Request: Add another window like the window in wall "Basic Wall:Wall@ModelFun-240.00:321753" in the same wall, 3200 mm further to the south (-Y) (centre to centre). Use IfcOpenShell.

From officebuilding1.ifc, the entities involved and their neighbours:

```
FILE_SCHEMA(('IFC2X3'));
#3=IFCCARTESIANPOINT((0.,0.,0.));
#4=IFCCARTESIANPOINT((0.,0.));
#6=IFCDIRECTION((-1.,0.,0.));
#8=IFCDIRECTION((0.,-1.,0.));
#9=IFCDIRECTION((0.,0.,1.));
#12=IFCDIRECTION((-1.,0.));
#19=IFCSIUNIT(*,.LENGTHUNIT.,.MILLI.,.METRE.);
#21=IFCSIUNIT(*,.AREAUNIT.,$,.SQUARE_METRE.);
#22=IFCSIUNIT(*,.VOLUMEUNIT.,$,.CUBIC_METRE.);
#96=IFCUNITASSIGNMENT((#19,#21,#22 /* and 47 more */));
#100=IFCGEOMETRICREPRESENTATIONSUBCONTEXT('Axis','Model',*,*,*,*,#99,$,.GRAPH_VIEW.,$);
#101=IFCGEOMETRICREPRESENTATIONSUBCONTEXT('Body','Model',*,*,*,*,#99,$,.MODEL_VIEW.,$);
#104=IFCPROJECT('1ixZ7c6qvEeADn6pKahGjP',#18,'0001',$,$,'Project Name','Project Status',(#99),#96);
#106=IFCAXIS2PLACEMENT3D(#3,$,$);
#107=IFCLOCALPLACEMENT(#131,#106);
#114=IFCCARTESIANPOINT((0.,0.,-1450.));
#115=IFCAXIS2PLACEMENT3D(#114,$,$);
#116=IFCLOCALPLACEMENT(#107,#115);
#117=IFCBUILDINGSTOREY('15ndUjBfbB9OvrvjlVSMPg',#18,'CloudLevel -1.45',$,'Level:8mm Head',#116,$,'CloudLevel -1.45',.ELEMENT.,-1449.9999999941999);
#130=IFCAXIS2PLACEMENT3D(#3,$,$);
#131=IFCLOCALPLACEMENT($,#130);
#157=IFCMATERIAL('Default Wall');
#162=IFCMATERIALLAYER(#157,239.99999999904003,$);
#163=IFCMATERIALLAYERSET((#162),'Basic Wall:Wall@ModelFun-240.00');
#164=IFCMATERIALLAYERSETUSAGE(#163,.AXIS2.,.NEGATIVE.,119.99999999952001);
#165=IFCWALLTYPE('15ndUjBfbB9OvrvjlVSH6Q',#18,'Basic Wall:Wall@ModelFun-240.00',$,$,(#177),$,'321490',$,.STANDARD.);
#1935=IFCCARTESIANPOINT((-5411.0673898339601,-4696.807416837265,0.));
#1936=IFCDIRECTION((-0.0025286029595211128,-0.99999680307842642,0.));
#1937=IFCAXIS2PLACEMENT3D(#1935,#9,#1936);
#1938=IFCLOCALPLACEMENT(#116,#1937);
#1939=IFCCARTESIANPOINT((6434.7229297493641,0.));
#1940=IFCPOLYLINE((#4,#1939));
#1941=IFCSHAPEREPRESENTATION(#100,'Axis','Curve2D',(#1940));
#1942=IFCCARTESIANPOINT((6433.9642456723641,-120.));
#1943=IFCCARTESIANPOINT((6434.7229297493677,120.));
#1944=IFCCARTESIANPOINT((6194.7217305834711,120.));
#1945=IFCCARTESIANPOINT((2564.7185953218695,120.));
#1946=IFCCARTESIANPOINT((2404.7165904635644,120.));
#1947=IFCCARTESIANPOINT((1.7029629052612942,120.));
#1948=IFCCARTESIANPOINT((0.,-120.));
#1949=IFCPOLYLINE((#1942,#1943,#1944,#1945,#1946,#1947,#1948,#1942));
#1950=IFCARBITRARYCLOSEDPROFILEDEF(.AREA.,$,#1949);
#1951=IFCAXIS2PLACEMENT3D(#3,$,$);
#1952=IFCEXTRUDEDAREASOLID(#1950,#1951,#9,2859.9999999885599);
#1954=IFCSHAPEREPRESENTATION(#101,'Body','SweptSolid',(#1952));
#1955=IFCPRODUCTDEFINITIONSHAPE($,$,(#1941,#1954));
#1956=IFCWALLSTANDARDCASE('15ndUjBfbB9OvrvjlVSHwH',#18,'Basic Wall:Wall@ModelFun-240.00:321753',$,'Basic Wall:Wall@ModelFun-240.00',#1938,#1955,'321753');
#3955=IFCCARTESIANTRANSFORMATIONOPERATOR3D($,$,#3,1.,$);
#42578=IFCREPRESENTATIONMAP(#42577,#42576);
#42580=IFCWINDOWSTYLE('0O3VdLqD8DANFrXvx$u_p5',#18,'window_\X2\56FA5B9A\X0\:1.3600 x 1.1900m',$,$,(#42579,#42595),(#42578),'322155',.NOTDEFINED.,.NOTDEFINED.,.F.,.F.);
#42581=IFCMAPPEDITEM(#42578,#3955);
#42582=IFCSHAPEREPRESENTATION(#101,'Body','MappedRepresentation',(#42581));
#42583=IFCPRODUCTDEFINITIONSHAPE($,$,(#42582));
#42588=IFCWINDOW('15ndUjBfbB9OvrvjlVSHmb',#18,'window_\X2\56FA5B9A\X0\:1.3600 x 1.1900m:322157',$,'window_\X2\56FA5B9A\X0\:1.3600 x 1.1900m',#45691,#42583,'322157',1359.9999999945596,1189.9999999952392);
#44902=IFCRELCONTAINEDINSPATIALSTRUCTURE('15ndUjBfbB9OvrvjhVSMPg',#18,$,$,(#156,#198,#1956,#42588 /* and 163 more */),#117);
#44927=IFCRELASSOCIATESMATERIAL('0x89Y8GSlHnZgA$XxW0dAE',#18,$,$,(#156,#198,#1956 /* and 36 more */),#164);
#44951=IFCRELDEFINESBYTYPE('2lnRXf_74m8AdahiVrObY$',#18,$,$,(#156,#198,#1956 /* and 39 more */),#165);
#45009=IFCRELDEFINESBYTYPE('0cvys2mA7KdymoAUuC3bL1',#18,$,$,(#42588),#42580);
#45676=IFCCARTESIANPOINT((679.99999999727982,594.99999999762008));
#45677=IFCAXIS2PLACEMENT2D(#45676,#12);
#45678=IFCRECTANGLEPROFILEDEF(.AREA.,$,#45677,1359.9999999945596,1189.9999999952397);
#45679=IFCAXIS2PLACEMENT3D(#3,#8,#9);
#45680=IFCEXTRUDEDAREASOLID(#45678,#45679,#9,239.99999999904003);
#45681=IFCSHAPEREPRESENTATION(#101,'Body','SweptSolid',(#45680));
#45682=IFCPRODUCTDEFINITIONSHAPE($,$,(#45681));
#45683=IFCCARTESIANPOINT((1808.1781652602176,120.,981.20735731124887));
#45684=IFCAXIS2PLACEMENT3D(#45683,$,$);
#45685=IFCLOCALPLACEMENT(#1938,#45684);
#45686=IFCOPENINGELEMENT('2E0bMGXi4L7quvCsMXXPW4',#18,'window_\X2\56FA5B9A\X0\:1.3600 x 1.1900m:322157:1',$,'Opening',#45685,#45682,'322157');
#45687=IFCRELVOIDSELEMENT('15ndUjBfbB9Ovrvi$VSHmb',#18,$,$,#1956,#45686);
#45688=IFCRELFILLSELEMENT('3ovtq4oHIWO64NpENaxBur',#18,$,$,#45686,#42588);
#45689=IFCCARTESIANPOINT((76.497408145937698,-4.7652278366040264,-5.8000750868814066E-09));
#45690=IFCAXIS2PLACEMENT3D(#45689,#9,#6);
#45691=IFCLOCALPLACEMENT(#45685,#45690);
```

```python
import ifcopenshell
import ifcopenshell.api.feature
import ifcopenshell.api.geometry
import ifcopenshell.api.root
import ifcopenshell.geom
import ifcopenshell.util.element
import ifcopenshell.util.placement
import ifcopenshell.util.shape
import ifcopenshell.util.unit

model = ifcopenshell.open("officebuilding1.ifc")
unit_scale = ifcopenshell.util.unit.calculate_unit_scale(model)
settings = ifcopenshell.geom.settings()


def volume(element):
    """Net volume in cubic metres, openings subtracted."""
    shape = ifcopenshell.geom.create_shape(settings, element)
    return ifcopenshell.util.shape.get_volume(shape.geometry)


def reuse_history(source, copy):
    """copy_class also copies each property set's owner history, people and application; keep the originals."""
    for rel in copy.IsDefinedBy:
        if rel.is_a("IfcRelDefinesByProperties") and (history := rel.RelatingPropertyDefinition.OwnerHistory):
            rel.RelatingPropertyDefinition.OwnerHistory = source.OwnerHistory
            ifcopenshell.util.element.remove_deep2(model, history)


window = model.by_guid("15ndUjBfbB9OvrvjlVSHmb")
opening = window.FillsVoids[0].RelatingOpeningElement
wall = opening.VoidsElements[0].RelatingBuildingElement
before = volume(wall)
shift = ifcopenshell.util.placement.get_local_placement(wall.ObjectPlacement)[:3, 0] * 3.2 / unit_scale

# copy_class copies the void relationship, type, container and properties, but no geometry.
new_opening = ifcopenshell.api.root.copy_class(model, product=opening)
new_opening.Representation = ifcopenshell.util.element.copy_deep(
    model, opening.Representation, exclude=["IfcGeometricRepresentationContext", "IfcRepresentationMap"]
)
new_opening.Name = "window_固定:1.3600 x 1.1900m"
new_opening.Tag = None
new_window = ifcopenshell.api.root.copy_class(model, product=window)
new_window.Representation = ifcopenshell.util.element.copy_deep(
    model, window.Representation, exclude=["IfcGeometricRepresentationContext", "IfcRepresentationMap"]
)
new_window.Name = "window_固定:1.3600 x 1.1900m"
new_window.Tag = None
reuse_history(window, new_window)
fills = ifcopenshell.api.feature.add_filling(model, opening=new_opening, element=new_window)
fills.OwnerHistory = new_window.OwnerHistory  # required in IFC2X3

for old, new in ((opening, new_opening), (window, new_window)):
    matrix = ifcopenshell.util.placement.get_local_placement(old.ObjectPlacement)
    matrix[:3, 3] += shift
    ifcopenshell.api.geometry.edit_object_placement(model, product=new, matrix=matrix, is_si=False)

after = volume(wall)

print(f"wall volume {before:.3f} -> {after:.3f} m3")

model.write("officebuilding1_edited.ifc")
```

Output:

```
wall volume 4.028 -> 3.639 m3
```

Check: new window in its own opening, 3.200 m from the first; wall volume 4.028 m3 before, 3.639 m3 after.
